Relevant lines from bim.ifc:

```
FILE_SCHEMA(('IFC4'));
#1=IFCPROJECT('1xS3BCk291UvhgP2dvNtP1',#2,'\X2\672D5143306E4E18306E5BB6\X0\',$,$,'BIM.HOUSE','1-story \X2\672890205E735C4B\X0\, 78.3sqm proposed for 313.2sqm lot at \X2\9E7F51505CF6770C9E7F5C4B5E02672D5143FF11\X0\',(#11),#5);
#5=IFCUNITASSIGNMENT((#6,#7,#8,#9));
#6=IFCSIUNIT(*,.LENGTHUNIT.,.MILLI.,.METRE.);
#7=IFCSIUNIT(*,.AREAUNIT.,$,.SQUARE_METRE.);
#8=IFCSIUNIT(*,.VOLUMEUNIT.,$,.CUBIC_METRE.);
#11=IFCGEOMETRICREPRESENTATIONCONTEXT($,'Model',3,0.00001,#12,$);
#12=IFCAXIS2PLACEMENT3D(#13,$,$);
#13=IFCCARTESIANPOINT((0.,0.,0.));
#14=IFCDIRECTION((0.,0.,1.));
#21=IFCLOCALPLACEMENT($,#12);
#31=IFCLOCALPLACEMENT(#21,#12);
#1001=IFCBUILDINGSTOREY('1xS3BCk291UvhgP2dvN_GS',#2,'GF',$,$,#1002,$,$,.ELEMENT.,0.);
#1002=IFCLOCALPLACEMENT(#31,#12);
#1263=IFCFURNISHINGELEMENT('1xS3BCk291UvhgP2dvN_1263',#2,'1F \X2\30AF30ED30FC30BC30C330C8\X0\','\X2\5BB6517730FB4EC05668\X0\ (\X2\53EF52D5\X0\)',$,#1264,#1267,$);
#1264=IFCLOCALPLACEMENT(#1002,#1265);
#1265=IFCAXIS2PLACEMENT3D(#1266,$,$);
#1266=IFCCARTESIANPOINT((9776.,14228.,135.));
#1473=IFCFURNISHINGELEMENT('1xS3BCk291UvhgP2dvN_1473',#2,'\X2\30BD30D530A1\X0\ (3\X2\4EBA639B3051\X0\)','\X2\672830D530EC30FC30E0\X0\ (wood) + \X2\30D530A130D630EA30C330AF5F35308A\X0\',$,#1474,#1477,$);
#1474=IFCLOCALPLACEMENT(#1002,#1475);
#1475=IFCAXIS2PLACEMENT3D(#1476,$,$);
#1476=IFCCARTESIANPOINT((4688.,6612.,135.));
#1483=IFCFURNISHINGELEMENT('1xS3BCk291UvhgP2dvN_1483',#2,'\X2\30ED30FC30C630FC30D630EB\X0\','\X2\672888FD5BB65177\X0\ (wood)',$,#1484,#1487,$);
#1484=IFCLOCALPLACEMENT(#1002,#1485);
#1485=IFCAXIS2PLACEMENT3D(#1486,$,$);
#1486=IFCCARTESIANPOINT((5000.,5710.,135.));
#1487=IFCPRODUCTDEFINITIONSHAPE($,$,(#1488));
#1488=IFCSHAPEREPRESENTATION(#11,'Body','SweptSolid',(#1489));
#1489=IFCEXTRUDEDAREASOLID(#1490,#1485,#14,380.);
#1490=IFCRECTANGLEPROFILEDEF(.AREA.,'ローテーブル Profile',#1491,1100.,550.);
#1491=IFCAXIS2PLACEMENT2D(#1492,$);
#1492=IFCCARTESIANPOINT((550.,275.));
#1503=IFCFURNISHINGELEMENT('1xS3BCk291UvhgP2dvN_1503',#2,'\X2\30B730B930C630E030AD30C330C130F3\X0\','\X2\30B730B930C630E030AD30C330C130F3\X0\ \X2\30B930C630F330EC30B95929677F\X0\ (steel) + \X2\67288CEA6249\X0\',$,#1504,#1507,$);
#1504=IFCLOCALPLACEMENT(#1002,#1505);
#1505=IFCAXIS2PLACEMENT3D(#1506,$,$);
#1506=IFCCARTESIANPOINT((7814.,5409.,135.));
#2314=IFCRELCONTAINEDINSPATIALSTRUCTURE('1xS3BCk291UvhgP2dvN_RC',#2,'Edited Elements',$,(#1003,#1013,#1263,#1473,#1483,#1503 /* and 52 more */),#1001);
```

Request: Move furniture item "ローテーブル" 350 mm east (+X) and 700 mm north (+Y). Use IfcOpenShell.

```python
import ifcopenshell
import ifcopenshell.api.geometry
import ifcopenshell.util.placement
import ifcopenshell.util.unit

model = ifcopenshell.open("bim.ifc")
unit_scale = ifcopenshell.util.unit.calculate_unit_scale(model)

item = model.by_guid("1xS3BCk291UvhgP2dvN_1483")
matrix = ifcopenshell.util.placement.get_local_placement(item.ObjectPlacement)
matrix[0, 3] += 0.35 / unit_scale
matrix[1, 3] += 0.7 / unit_scale
ifcopenshell.api.geometry.edit_object_placement(model, product=item, matrix=matrix, is_si=False)

print(ifcopenshell.util.placement.get_local_placement(item.ObjectPlacement).round(3) + 0.0)

model.write("bim_updated.ifc")
```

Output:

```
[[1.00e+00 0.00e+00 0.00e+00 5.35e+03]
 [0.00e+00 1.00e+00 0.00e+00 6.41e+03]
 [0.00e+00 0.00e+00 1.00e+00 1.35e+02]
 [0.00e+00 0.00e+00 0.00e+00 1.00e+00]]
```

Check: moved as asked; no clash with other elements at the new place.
